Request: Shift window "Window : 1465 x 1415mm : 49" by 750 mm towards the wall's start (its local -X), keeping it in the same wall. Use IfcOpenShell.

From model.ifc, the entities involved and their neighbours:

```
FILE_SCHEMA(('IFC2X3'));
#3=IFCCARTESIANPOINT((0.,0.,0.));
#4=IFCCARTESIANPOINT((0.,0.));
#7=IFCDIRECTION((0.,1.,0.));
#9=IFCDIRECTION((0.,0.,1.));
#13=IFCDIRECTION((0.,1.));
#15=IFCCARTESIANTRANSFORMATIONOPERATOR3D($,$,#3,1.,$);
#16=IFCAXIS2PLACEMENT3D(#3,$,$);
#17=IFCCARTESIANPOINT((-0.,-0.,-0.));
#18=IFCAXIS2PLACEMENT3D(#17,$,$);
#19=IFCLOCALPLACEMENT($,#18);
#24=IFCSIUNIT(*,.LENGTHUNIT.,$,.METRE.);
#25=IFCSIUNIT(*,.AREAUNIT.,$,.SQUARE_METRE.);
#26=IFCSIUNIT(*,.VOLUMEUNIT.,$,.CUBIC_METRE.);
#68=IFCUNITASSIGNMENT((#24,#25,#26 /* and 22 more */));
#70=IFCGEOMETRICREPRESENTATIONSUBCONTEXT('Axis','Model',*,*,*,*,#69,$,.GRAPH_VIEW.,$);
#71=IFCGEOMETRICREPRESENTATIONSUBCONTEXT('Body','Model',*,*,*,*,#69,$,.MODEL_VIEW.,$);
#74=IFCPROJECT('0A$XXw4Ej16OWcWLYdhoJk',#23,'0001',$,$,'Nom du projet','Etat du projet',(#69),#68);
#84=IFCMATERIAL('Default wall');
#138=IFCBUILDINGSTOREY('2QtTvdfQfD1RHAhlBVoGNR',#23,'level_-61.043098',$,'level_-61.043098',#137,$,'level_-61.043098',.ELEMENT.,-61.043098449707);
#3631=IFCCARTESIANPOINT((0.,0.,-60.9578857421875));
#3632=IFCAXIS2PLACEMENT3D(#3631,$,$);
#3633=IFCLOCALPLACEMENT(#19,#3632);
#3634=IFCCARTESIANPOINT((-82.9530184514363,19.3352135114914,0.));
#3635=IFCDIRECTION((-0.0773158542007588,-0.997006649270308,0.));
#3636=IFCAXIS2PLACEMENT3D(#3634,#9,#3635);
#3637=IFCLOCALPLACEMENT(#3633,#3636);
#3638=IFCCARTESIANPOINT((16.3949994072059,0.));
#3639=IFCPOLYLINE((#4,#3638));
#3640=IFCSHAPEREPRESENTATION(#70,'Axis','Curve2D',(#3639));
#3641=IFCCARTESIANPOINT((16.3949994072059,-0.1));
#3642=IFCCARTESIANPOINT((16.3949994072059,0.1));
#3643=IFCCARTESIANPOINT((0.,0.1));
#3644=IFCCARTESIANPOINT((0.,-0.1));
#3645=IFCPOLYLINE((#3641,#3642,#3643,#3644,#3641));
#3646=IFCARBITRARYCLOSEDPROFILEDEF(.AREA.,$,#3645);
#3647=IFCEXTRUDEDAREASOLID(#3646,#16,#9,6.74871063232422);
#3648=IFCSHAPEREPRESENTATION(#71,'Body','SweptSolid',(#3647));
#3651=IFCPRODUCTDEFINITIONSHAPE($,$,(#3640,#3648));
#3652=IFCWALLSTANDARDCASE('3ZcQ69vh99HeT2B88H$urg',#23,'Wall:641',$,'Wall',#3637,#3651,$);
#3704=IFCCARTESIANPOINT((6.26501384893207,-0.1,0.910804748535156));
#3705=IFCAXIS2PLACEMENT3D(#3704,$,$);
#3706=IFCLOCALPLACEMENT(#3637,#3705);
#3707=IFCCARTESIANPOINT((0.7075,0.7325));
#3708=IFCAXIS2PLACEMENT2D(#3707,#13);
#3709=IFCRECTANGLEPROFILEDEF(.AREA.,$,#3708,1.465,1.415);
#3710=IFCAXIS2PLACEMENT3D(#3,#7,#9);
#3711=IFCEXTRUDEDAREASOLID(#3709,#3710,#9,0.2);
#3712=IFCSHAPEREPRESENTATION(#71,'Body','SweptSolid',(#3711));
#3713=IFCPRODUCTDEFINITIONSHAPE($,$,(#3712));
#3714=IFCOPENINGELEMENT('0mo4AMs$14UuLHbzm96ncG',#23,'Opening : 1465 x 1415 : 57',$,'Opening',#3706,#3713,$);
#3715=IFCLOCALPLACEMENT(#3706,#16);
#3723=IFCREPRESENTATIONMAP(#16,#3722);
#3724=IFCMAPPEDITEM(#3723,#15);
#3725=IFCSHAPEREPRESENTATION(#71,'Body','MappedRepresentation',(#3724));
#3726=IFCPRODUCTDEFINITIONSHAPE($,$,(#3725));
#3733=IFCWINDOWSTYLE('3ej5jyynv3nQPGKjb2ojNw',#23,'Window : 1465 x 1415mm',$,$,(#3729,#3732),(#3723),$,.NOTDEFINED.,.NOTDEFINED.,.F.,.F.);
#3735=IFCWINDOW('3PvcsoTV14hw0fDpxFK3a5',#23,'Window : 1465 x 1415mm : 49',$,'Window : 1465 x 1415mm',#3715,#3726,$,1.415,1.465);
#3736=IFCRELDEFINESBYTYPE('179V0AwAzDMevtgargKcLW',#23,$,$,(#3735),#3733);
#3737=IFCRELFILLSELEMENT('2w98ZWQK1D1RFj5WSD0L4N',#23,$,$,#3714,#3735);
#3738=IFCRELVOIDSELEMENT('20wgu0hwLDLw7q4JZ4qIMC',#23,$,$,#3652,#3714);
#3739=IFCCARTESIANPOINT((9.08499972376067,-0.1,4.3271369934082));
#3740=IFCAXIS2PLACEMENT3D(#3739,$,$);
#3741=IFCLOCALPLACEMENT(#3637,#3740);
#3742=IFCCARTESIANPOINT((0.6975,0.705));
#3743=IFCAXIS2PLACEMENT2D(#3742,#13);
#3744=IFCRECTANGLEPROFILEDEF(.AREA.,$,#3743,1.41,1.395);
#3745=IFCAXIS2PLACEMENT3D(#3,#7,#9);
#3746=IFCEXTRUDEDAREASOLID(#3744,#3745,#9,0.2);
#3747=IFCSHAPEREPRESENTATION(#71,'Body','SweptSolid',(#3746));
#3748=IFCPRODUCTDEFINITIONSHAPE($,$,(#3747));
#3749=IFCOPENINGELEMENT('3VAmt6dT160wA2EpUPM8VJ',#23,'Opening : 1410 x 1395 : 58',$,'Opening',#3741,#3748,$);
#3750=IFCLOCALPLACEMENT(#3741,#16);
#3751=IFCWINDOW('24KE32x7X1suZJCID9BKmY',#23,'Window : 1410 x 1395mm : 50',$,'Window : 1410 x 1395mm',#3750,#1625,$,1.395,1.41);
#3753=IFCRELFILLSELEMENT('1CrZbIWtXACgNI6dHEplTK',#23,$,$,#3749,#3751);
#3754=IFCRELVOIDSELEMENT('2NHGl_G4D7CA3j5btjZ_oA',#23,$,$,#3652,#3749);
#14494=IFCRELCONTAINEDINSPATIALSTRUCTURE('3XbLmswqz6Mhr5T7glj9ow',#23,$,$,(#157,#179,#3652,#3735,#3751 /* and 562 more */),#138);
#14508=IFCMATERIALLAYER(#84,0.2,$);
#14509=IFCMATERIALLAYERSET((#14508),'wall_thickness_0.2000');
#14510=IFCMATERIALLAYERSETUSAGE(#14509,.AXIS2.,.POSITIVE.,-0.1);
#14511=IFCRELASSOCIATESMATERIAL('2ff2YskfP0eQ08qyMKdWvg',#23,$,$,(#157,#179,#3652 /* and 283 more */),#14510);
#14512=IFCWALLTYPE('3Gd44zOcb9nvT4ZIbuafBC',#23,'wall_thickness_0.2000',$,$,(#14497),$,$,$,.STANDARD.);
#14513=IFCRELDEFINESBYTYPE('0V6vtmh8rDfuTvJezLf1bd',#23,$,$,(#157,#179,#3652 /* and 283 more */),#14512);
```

```python
import ifcopenshell
import ifcopenshell.api.geometry
import ifcopenshell.util.placement
import ifcopenshell.util.unit

model = ifcopenshell.open("model.ifc")
unit_scale = ifcopenshell.util.unit.calculate_unit_scale(model)

window = model.by_guid("3PvcsoTV14hw0fDpxFK3a5")
opening = window.FillsVoids[0].RelatingOpeningElement
wall = opening.VoidsElements[0].RelatingBuildingElement

wall_matrix = ifcopenshell.util.placement.get_local_placement(wall.ObjectPlacement)
shift = wall_matrix[:3, 0] * -0.75 / unit_scale
before = ifcopenshell.util.placement.get_local_placement(window.ObjectPlacement)[:3, 3].copy()

# The window is placed relative to its opening, so it follows when the opening moves.
matrix = ifcopenshell.util.placement.get_local_placement(opening.ObjectPlacement)
matrix[:3, 3] += shift
ifcopenshell.api.geometry.edit_object_placement(
    model, product=opening, matrix=matrix, is_si=False, should_transform_children=True
)

after = ifcopenshell.util.placement.get_local_placement(window.ObjectPlacement)[:3, 3]
print("window moved by", (after - before).round(3) + 0.0)

model.write("model-out.ifc")
```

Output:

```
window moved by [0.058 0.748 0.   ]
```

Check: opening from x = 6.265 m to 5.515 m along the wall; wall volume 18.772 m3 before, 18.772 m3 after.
